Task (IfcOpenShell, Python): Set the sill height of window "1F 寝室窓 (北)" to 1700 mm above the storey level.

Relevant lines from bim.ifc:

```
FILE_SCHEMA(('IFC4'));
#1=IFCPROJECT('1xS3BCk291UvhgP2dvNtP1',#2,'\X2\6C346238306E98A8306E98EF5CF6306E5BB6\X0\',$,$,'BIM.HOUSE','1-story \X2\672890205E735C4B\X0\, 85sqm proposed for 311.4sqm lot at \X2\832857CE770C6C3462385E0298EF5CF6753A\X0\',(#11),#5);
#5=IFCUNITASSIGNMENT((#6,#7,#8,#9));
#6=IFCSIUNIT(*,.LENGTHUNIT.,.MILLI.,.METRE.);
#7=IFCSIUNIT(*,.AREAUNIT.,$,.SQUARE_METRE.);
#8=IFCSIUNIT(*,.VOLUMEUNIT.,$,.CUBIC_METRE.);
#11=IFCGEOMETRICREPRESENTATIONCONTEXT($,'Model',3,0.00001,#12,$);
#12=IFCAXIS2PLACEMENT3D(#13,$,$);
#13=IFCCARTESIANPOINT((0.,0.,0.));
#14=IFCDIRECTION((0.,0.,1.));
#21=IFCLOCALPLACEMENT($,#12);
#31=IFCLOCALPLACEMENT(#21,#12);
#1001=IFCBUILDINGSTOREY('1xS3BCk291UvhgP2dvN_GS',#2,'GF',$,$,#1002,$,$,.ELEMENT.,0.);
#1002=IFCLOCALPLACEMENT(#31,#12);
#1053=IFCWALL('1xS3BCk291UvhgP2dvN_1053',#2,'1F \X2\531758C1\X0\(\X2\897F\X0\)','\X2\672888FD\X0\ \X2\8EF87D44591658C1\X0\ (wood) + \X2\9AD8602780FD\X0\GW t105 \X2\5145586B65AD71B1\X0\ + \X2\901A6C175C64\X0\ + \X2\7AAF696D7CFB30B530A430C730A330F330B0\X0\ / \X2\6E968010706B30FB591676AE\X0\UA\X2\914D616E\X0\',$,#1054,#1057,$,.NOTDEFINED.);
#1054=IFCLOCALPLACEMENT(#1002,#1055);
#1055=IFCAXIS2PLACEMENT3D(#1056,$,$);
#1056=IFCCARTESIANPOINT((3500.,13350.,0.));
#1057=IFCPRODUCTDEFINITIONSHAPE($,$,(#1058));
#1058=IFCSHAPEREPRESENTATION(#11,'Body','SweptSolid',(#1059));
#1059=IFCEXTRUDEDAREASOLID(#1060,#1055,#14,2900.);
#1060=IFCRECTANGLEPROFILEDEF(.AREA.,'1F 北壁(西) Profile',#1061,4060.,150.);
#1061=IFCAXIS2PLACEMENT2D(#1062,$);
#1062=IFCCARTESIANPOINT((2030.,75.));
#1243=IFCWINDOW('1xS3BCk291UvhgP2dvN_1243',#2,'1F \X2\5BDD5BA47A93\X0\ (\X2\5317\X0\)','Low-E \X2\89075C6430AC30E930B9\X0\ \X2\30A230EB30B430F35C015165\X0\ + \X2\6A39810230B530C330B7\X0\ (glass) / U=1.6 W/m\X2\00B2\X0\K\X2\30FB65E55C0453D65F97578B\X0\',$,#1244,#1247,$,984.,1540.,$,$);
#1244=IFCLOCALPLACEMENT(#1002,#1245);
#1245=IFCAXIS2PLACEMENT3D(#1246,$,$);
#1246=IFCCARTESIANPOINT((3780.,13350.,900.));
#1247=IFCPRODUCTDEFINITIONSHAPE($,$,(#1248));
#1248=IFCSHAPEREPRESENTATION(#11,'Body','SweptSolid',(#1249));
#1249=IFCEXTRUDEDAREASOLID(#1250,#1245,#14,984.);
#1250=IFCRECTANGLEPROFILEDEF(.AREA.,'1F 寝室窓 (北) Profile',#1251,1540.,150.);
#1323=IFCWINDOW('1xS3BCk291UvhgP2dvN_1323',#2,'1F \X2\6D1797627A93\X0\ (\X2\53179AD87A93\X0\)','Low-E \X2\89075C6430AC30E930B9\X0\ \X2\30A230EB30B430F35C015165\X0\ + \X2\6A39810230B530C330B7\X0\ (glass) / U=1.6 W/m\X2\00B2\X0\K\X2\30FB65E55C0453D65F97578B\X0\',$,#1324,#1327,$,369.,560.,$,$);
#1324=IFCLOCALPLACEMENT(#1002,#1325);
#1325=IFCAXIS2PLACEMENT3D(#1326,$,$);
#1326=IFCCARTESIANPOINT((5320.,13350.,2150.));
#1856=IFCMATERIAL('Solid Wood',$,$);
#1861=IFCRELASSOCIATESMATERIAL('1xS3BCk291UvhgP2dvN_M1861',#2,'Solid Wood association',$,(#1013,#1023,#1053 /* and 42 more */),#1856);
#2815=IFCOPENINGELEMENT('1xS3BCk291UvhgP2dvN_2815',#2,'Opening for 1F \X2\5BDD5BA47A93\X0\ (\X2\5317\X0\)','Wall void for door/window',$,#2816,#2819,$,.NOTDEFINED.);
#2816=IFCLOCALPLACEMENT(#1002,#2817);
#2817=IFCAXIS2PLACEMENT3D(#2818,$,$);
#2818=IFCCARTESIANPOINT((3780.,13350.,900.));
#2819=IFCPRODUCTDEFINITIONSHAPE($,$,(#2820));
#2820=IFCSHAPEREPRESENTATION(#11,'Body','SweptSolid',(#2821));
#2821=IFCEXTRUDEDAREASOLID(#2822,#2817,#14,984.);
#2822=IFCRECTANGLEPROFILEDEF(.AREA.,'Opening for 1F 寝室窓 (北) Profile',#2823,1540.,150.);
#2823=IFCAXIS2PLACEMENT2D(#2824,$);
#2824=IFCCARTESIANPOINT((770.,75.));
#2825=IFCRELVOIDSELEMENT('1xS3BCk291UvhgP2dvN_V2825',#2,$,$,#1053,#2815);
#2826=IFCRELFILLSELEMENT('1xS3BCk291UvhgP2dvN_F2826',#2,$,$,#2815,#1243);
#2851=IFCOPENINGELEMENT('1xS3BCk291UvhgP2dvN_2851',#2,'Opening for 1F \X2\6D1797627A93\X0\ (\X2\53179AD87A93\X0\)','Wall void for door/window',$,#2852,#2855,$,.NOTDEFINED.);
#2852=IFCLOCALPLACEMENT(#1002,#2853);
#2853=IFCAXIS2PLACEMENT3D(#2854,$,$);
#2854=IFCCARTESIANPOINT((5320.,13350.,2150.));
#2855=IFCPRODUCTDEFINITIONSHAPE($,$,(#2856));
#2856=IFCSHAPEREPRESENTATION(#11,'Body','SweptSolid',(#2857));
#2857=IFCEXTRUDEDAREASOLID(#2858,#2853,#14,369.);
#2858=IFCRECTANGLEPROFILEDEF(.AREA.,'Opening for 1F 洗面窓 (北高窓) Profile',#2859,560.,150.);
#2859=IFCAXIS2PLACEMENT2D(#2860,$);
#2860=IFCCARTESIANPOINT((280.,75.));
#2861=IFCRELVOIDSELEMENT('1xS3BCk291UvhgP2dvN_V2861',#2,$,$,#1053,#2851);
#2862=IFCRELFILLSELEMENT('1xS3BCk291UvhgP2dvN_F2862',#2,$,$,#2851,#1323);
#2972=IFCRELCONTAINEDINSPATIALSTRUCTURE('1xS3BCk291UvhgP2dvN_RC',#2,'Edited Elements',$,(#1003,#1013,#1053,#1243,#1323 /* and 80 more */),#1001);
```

```python
import numpy as np
import ifcopenshell
import ifcopenshell.api.geometry
import ifcopenshell.geom
import ifcopenshell.util.element
import ifcopenshell.util.placement
import ifcopenshell.util.shape
import ifcopenshell.util.unit

model = ifcopenshell.open("bim.ifc")
unit_scale = ifcopenshell.util.unit.calculate_unit_scale(model)

window = model.by_guid("1xS3BCk291UvhgP2dvN_1243")
opening = window.FillsVoids[0].RelatingOpeningElement
storey = ifcopenshell.util.element.get_container(window, ifc_class="IfcBuildingStorey")
level = ifcopenshell.util.placement.get_local_placement(storey.ObjectPlacement)[2, 3]

# The opening's origin need not be at the sill, so measure its lowest point.
shape = ifcopenshell.geom.create_shape(ifcopenshell.geom.settings(), opening)
bottom = ifcopenshell.util.shape.get_shape_bottom_elevation(shape, shape.geometry) / unit_scale
dz = level + 1.7 / unit_scale - bottom

shift = np.array([0.0, 0.0, dz])
# The window is not placed relative to its opening, so move both.
for product in (opening, window):
    matrix = ifcopenshell.util.placement.get_local_placement(product.ObjectPlacement)
    matrix[:3, 3] += shift
    ifcopenshell.api.geometry.edit_object_placement(model, product=product, matrix=matrix, is_si=False)

print(f"moved by {dz * unit_scale:+.3f} m")

model.write("bim-out.ifc")
```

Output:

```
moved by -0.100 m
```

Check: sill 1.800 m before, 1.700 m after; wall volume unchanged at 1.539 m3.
